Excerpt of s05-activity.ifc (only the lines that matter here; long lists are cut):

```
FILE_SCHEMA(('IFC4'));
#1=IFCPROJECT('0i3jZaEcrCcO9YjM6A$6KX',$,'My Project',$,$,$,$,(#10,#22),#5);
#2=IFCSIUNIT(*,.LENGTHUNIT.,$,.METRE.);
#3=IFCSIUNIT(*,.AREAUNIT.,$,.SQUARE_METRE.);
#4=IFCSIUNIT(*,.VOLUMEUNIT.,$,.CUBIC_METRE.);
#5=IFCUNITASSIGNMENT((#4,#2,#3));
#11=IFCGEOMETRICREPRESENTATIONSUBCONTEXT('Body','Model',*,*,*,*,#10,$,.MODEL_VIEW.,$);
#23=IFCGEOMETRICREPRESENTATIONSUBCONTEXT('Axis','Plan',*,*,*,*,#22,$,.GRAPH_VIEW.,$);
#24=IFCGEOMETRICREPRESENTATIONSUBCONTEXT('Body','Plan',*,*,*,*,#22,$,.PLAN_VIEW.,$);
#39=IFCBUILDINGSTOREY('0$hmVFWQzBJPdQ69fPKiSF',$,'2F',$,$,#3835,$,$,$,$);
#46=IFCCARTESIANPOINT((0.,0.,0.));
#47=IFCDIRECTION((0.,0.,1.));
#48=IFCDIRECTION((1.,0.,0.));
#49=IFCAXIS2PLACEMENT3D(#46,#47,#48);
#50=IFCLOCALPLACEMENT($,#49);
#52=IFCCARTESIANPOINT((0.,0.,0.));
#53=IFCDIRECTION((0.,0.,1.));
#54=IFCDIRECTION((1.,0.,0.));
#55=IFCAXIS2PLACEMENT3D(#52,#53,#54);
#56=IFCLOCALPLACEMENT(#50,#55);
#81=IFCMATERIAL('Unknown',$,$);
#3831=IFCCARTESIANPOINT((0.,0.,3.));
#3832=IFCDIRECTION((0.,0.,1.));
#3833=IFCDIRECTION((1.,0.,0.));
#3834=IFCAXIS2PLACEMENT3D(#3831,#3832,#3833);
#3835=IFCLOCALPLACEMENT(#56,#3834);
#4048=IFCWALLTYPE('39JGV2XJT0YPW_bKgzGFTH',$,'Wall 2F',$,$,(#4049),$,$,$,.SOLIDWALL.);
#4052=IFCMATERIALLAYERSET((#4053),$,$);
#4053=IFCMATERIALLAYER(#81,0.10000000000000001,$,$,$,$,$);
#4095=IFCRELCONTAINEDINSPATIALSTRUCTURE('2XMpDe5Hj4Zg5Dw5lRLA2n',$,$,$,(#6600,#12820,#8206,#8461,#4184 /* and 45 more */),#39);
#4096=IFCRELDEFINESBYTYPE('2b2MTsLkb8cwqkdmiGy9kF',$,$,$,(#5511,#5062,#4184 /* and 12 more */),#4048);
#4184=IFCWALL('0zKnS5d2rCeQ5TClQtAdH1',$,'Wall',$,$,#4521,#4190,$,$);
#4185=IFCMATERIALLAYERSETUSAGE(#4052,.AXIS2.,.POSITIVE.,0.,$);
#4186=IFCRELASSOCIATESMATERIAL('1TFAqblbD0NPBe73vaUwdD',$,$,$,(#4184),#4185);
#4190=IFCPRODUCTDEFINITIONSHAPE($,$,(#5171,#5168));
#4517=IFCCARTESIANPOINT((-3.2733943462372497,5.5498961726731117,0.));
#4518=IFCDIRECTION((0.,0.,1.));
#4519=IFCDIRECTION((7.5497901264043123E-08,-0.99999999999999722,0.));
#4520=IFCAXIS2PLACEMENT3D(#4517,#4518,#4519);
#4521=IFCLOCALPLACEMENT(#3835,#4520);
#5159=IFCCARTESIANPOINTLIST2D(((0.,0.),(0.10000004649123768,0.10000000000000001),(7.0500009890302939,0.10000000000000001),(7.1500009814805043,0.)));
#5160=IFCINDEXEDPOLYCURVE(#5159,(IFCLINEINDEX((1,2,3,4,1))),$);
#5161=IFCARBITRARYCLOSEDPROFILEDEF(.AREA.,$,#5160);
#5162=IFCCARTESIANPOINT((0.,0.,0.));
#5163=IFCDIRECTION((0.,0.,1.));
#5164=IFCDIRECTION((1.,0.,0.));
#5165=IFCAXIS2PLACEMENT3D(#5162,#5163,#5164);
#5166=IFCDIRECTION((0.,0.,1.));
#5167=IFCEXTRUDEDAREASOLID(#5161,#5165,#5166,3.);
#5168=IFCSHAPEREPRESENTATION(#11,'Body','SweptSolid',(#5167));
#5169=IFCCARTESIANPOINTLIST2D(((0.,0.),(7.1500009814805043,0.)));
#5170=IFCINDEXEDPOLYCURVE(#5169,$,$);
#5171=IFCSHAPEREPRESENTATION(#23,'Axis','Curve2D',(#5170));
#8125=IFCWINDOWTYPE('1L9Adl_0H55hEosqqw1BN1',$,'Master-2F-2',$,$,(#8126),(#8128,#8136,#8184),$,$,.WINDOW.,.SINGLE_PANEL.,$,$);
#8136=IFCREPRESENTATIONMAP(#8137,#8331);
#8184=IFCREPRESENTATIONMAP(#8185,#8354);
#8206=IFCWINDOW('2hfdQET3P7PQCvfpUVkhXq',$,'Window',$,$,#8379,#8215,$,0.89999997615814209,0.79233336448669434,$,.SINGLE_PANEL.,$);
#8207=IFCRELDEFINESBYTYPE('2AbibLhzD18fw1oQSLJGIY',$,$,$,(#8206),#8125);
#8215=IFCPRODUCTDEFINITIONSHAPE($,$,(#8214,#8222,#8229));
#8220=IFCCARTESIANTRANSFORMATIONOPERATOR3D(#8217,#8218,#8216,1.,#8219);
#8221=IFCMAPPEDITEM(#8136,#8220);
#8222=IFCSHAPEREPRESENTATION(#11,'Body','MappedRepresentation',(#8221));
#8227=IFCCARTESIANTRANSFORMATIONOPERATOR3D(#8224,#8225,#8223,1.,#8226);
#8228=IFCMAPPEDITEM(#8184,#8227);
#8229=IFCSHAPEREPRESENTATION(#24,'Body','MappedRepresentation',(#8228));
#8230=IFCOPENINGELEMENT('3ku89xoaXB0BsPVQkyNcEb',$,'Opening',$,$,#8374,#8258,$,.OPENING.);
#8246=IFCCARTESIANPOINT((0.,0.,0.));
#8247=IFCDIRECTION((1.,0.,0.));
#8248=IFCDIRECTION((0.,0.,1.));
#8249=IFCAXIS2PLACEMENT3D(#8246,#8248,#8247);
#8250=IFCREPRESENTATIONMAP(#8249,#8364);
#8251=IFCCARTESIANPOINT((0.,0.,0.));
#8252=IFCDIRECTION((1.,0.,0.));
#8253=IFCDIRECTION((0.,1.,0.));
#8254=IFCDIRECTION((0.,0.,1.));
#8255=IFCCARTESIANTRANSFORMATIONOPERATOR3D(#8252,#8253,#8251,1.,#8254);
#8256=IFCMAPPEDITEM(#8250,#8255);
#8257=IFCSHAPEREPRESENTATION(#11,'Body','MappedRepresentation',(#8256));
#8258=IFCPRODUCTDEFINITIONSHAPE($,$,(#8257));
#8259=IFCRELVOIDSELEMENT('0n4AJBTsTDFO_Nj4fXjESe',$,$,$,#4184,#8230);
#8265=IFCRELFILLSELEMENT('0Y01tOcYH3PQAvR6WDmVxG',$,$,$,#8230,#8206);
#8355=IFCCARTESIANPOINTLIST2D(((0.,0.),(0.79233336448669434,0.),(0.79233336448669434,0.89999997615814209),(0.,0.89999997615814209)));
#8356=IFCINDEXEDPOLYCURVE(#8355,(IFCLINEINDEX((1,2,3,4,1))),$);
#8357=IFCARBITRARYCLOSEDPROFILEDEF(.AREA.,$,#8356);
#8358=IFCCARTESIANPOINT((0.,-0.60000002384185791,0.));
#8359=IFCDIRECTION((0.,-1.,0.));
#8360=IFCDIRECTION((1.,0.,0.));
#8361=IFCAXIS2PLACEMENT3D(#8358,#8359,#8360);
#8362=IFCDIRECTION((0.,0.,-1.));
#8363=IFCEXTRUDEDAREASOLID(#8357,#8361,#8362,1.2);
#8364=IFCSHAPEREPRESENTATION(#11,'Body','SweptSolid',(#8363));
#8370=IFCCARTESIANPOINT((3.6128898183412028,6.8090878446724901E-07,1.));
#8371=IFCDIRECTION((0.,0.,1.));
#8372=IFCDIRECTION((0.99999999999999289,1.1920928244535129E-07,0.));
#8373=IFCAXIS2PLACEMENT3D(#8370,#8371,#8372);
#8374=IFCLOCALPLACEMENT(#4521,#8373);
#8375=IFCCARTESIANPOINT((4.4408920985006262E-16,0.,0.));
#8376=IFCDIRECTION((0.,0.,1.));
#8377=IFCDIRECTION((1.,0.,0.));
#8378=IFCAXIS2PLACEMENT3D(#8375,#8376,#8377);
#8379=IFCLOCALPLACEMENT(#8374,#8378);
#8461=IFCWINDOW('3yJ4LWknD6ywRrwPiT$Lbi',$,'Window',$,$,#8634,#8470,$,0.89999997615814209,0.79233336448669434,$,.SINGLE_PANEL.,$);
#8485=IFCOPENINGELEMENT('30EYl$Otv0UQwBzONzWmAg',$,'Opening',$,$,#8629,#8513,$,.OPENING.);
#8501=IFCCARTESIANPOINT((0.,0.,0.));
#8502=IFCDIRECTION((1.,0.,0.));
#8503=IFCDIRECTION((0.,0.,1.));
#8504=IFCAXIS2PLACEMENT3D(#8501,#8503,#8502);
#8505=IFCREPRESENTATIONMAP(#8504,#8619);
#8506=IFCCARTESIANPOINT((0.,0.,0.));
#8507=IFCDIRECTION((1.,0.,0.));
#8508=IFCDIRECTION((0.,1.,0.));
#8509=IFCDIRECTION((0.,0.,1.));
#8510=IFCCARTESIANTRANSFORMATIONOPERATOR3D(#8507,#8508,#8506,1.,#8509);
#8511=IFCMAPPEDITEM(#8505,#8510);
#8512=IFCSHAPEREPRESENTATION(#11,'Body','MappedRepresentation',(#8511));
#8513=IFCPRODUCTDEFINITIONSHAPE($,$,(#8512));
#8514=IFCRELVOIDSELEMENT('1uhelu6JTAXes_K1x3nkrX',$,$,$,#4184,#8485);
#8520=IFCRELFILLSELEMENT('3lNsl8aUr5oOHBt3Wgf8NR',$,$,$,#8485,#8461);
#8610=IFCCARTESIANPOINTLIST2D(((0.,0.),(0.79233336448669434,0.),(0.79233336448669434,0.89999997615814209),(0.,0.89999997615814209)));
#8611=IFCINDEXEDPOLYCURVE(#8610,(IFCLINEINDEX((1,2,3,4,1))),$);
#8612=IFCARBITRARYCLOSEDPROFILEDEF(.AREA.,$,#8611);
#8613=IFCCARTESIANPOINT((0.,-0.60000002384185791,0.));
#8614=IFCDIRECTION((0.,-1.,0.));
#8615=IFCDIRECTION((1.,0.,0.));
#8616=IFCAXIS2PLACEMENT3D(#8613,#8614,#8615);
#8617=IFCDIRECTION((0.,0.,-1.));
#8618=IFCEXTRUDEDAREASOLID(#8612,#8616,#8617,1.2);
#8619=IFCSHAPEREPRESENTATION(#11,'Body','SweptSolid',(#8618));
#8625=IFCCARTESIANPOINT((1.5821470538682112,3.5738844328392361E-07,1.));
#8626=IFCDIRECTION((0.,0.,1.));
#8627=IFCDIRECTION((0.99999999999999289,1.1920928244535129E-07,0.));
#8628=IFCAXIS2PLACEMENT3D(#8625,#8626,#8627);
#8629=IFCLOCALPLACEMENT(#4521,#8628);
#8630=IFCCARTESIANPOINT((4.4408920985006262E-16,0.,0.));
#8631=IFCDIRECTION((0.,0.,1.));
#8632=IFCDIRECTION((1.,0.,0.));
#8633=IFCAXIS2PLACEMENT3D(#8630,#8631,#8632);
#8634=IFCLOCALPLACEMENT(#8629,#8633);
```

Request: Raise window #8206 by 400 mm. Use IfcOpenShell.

```python
import numpy as np
import ifcopenshell
import ifcopenshell.api.geometry
import ifcopenshell.util.placement
import ifcopenshell.util.unit

model = ifcopenshell.open("s05-activity.ifc")
unit_scale = ifcopenshell.util.unit.calculate_unit_scale(model)

window = model.by_id(8206)
opening = window.FillsVoids[0].RelatingOpeningElement
dz = 0.4

shift = np.array([0.0, 0.0, dz])
# The window is placed relative to its opening, so it follows when the opening moves.
matrix = ifcopenshell.util.placement.get_local_placement(opening.ObjectPlacement)
matrix[:3, 3] += shift
ifcopenshell.api.geometry.edit_object_placement(
    model, product=opening, matrix=matrix, is_si=False, should_transform_children=True
)

print(f"moved by {dz * unit_scale:+.3f} m")

model.write("s05-activity_updated.ifc")
```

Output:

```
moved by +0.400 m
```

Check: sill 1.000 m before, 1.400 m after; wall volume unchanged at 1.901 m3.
